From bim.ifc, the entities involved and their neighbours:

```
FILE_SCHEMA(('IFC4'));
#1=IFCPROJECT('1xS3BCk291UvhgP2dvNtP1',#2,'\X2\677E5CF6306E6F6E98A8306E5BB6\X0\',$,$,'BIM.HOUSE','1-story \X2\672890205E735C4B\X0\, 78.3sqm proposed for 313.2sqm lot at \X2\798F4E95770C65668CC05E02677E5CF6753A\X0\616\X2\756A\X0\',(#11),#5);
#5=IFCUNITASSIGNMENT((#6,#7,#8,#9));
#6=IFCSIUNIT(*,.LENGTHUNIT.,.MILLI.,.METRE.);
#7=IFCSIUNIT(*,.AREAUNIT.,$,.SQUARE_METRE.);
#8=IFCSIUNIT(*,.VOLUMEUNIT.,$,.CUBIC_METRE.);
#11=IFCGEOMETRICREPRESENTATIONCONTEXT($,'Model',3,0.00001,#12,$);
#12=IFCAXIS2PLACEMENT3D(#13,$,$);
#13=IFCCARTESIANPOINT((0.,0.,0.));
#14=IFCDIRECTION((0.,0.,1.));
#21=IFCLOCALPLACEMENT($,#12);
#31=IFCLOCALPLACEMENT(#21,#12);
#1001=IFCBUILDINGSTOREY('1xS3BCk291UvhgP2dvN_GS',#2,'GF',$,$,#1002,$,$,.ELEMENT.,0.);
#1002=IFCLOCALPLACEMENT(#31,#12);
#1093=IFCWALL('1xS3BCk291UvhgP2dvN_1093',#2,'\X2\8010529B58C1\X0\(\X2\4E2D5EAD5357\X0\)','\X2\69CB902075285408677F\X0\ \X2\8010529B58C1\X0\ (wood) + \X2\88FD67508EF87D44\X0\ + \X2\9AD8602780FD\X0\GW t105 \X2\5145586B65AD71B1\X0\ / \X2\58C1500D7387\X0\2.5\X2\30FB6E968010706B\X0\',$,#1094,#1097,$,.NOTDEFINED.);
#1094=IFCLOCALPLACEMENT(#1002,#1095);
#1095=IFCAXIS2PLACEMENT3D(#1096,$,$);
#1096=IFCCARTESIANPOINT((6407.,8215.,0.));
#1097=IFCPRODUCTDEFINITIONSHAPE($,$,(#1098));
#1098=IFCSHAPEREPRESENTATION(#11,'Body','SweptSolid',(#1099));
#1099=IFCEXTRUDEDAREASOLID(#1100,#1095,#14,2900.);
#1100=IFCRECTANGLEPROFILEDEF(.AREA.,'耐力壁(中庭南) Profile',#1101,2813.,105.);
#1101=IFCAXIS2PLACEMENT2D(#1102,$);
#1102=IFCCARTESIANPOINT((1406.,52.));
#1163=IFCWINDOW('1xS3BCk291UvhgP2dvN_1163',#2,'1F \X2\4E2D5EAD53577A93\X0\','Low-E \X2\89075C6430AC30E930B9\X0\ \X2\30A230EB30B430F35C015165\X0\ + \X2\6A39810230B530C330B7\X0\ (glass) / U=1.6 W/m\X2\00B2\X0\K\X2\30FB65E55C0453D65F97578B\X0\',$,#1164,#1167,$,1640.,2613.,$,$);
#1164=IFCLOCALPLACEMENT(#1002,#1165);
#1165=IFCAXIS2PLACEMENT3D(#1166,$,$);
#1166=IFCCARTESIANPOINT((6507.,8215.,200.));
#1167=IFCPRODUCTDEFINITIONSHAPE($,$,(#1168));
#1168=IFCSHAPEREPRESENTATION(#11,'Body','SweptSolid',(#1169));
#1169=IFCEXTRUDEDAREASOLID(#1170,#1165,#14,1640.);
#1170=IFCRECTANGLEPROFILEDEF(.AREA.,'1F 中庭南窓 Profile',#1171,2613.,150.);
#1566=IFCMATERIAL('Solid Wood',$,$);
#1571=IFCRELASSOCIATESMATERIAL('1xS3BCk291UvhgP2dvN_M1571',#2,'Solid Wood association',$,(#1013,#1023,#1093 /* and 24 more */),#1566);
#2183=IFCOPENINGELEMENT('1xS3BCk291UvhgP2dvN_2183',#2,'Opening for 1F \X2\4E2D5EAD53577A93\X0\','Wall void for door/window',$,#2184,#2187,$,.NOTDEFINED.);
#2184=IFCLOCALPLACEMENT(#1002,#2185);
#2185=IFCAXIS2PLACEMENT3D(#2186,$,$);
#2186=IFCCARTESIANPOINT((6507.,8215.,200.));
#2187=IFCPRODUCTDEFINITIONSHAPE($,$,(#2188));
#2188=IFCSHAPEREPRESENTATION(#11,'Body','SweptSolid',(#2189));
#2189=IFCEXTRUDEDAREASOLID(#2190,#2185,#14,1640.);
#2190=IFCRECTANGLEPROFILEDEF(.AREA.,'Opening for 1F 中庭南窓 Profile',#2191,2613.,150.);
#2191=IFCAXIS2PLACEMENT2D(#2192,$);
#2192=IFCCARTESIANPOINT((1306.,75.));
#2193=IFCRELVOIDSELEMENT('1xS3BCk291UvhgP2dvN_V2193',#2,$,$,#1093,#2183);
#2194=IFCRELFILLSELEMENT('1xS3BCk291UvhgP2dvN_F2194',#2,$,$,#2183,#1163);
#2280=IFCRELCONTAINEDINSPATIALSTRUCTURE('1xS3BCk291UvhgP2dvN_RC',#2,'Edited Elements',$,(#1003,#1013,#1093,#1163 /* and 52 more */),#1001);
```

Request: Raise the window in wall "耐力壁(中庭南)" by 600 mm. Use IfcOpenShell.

```python
import numpy as np
import ifcopenshell
import ifcopenshell.api.geometry
import ifcopenshell.util.placement
import ifcopenshell.util.unit

model = ifcopenshell.open("bim.ifc")
unit_scale = ifcopenshell.util.unit.calculate_unit_scale(model)

window = model.by_guid("1xS3BCk291UvhgP2dvN_1163")
opening = window.FillsVoids[0].RelatingOpeningElement
dz = 600.0

shift = np.array([0.0, 0.0, dz])
# The window is not placed relative to its opening, so move both.
for product in (opening, window):
    matrix = ifcopenshell.util.placement.get_local_placement(product.ObjectPlacement)
    matrix[:3, 3] += shift
    ifcopenshell.api.geometry.edit_object_placement(model, product=product, matrix=matrix, is_si=False)

print(f"moved by {dz * unit_scale:+.3f} m")

model.write("bim_rev.ifc")
```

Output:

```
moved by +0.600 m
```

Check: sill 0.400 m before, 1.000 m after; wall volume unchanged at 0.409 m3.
